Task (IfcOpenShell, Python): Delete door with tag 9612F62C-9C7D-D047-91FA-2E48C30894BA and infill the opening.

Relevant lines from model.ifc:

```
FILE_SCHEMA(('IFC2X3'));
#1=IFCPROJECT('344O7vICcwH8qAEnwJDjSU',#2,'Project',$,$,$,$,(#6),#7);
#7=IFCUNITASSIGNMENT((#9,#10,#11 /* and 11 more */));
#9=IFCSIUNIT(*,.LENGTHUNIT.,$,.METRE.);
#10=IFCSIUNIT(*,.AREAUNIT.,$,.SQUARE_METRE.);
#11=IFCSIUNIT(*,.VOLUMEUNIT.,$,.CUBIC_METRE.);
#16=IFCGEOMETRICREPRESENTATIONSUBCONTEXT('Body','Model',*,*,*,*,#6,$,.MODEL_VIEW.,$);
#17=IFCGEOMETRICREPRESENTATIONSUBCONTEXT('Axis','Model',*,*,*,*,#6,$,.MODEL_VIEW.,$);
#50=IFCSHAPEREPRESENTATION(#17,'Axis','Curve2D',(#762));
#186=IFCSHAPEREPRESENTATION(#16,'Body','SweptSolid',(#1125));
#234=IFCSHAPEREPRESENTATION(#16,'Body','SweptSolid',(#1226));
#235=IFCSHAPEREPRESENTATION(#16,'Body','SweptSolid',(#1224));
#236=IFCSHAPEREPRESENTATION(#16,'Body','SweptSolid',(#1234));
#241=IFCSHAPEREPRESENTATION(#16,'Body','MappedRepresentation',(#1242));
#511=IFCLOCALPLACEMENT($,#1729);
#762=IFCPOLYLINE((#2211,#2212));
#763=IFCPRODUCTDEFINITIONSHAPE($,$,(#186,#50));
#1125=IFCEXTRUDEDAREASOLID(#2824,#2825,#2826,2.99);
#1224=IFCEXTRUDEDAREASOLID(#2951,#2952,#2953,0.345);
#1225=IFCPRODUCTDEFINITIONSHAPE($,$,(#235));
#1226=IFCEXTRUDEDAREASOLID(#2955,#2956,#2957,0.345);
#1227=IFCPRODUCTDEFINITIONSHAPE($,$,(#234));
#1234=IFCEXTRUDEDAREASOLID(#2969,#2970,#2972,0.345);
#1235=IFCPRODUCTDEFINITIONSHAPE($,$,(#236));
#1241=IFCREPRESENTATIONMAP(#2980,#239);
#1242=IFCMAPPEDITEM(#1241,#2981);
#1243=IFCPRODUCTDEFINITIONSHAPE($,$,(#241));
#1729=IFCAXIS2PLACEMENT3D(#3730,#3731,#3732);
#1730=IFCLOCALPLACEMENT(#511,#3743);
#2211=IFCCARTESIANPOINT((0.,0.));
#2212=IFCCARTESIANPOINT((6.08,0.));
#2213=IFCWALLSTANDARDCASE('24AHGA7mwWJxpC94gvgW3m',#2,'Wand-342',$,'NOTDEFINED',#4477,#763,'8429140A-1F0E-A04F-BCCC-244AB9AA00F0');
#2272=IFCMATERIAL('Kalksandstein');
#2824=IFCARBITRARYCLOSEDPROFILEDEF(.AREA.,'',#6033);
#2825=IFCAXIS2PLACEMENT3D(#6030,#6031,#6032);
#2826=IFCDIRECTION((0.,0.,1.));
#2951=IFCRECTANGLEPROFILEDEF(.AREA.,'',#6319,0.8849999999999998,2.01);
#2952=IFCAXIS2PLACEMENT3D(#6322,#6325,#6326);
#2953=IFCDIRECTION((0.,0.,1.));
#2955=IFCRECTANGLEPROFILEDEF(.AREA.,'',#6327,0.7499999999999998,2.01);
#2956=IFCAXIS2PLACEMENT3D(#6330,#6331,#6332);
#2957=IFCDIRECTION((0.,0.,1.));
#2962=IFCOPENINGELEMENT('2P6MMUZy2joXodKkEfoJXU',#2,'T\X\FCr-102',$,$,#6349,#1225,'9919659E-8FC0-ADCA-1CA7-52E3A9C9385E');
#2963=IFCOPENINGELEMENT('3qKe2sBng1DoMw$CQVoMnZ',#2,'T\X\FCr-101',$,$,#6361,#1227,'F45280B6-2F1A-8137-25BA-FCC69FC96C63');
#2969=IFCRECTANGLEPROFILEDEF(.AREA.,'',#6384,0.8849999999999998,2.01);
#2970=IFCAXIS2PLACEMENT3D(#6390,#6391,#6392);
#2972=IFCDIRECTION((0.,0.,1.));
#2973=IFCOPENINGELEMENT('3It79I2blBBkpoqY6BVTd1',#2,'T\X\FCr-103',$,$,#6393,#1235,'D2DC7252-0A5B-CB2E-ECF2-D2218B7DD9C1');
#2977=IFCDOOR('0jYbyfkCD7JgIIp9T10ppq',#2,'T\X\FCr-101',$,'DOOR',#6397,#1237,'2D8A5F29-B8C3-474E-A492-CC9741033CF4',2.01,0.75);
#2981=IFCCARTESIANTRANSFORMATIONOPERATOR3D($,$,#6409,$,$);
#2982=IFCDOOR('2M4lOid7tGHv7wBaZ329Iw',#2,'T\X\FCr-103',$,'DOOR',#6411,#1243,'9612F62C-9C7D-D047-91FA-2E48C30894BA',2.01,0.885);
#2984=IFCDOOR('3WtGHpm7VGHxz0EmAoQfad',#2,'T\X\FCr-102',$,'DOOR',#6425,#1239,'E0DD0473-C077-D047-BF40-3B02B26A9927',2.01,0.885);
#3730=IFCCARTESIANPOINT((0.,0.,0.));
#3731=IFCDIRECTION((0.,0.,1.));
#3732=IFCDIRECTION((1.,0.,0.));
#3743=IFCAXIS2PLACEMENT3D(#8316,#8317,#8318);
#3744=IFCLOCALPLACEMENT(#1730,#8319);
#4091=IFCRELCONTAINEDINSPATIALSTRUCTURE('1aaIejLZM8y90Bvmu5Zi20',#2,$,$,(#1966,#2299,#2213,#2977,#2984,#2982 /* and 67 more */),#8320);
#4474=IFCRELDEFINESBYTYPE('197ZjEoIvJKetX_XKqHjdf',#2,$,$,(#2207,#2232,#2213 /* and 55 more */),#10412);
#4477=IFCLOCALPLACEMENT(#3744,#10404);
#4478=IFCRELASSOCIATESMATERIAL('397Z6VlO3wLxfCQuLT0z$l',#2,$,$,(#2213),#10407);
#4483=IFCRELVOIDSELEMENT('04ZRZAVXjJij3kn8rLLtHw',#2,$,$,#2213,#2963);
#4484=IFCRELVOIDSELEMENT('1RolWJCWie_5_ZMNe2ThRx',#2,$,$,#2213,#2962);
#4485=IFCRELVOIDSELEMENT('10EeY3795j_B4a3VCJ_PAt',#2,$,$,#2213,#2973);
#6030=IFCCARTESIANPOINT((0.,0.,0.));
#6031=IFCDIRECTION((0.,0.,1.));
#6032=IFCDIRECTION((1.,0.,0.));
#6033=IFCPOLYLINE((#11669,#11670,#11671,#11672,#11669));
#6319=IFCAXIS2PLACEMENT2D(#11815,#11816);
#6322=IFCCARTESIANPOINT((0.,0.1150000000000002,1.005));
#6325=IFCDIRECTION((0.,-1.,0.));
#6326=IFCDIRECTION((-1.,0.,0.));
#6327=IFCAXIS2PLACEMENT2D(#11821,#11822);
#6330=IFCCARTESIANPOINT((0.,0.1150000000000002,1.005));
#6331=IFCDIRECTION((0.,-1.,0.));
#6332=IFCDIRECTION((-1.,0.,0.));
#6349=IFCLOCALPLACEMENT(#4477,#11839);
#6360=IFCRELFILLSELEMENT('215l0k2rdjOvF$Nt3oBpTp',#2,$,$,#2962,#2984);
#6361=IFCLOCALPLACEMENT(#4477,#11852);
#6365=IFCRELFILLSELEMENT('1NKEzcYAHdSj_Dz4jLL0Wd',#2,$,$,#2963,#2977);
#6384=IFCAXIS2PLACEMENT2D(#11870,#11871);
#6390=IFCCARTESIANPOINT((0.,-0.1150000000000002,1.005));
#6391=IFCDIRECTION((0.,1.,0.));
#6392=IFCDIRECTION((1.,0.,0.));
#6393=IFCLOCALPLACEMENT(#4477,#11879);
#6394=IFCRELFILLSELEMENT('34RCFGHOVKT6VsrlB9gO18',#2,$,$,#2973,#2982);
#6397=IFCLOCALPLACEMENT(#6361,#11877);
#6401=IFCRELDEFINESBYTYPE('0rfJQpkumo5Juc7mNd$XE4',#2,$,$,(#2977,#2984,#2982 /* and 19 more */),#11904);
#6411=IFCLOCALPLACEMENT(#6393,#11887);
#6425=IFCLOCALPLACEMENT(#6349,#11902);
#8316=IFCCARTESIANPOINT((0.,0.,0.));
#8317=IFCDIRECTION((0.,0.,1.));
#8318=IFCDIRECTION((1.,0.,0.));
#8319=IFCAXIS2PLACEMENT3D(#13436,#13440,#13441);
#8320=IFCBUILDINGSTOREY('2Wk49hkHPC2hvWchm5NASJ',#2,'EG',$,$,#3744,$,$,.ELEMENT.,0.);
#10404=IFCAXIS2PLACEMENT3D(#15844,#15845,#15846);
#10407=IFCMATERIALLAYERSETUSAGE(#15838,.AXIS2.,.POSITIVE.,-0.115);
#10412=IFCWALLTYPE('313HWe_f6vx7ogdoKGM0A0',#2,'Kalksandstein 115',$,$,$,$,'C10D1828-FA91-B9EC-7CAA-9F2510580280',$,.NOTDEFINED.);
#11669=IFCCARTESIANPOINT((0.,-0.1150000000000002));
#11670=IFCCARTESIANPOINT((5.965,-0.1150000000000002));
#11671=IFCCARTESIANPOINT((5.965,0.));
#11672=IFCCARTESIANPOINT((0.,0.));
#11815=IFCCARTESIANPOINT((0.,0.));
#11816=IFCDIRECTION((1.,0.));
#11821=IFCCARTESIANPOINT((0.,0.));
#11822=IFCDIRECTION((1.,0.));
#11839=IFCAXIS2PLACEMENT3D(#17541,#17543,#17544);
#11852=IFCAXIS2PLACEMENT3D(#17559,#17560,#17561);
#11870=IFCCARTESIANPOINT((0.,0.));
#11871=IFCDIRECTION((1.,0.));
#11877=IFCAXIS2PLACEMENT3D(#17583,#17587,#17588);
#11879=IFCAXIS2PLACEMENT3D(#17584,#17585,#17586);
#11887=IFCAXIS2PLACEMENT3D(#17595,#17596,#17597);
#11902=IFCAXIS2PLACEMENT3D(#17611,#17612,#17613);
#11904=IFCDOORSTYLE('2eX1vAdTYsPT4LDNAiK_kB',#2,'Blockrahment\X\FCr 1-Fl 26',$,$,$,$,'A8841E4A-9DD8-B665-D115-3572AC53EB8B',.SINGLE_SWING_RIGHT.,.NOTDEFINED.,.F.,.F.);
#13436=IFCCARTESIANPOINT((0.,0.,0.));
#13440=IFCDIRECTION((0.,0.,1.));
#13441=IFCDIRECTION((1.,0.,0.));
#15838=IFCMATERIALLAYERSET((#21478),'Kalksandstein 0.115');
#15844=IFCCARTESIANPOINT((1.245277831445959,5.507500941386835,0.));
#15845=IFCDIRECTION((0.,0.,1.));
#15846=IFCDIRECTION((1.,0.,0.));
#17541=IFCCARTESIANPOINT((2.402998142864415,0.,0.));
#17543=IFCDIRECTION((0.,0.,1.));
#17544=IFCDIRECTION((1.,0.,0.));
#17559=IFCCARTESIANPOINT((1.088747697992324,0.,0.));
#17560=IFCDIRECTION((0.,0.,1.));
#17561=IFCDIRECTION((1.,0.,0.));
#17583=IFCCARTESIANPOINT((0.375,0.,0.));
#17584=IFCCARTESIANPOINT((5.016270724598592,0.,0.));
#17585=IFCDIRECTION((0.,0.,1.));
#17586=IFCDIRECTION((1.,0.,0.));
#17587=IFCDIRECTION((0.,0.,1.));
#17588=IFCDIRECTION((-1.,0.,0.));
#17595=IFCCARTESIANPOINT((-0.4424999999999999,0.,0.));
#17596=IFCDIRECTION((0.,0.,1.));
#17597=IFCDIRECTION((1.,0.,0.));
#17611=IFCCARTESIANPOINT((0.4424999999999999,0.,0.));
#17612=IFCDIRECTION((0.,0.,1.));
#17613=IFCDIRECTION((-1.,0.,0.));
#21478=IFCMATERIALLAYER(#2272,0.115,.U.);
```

```python
import ifcopenshell
import ifcopenshell.api.feature
import ifcopenshell.api.root
import ifcopenshell.geom
import ifcopenshell.util.shape

model = ifcopenshell.open("model.ifc")
settings = ifcopenshell.geom.settings()


def volume(element):
    """Net volume in cubic metres, openings subtracted."""
    shape = ifcopenshell.geom.create_shape(settings, element)
    return ifcopenshell.util.shape.get_volume(shape.geometry)


door = model.by_guid("2M4lOid7tGHv7wBaZ329Iw")
opening = door.FillsVoids[0].RelatingOpeningElement
wall = opening.VoidsElements[0].RelatingBuildingElement
before = volume(wall)

ifcopenshell.api.root.remove_product(model, product=door)
ifcopenshell.api.feature.remove_feature(model, feature=opening)

after = volume(wall)

print(f"wall volume {before:.3f} -> {after:.3f} m3")

model.write("model_edited.ifc")
```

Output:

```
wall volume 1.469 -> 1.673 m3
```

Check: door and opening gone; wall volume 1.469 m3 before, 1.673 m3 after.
